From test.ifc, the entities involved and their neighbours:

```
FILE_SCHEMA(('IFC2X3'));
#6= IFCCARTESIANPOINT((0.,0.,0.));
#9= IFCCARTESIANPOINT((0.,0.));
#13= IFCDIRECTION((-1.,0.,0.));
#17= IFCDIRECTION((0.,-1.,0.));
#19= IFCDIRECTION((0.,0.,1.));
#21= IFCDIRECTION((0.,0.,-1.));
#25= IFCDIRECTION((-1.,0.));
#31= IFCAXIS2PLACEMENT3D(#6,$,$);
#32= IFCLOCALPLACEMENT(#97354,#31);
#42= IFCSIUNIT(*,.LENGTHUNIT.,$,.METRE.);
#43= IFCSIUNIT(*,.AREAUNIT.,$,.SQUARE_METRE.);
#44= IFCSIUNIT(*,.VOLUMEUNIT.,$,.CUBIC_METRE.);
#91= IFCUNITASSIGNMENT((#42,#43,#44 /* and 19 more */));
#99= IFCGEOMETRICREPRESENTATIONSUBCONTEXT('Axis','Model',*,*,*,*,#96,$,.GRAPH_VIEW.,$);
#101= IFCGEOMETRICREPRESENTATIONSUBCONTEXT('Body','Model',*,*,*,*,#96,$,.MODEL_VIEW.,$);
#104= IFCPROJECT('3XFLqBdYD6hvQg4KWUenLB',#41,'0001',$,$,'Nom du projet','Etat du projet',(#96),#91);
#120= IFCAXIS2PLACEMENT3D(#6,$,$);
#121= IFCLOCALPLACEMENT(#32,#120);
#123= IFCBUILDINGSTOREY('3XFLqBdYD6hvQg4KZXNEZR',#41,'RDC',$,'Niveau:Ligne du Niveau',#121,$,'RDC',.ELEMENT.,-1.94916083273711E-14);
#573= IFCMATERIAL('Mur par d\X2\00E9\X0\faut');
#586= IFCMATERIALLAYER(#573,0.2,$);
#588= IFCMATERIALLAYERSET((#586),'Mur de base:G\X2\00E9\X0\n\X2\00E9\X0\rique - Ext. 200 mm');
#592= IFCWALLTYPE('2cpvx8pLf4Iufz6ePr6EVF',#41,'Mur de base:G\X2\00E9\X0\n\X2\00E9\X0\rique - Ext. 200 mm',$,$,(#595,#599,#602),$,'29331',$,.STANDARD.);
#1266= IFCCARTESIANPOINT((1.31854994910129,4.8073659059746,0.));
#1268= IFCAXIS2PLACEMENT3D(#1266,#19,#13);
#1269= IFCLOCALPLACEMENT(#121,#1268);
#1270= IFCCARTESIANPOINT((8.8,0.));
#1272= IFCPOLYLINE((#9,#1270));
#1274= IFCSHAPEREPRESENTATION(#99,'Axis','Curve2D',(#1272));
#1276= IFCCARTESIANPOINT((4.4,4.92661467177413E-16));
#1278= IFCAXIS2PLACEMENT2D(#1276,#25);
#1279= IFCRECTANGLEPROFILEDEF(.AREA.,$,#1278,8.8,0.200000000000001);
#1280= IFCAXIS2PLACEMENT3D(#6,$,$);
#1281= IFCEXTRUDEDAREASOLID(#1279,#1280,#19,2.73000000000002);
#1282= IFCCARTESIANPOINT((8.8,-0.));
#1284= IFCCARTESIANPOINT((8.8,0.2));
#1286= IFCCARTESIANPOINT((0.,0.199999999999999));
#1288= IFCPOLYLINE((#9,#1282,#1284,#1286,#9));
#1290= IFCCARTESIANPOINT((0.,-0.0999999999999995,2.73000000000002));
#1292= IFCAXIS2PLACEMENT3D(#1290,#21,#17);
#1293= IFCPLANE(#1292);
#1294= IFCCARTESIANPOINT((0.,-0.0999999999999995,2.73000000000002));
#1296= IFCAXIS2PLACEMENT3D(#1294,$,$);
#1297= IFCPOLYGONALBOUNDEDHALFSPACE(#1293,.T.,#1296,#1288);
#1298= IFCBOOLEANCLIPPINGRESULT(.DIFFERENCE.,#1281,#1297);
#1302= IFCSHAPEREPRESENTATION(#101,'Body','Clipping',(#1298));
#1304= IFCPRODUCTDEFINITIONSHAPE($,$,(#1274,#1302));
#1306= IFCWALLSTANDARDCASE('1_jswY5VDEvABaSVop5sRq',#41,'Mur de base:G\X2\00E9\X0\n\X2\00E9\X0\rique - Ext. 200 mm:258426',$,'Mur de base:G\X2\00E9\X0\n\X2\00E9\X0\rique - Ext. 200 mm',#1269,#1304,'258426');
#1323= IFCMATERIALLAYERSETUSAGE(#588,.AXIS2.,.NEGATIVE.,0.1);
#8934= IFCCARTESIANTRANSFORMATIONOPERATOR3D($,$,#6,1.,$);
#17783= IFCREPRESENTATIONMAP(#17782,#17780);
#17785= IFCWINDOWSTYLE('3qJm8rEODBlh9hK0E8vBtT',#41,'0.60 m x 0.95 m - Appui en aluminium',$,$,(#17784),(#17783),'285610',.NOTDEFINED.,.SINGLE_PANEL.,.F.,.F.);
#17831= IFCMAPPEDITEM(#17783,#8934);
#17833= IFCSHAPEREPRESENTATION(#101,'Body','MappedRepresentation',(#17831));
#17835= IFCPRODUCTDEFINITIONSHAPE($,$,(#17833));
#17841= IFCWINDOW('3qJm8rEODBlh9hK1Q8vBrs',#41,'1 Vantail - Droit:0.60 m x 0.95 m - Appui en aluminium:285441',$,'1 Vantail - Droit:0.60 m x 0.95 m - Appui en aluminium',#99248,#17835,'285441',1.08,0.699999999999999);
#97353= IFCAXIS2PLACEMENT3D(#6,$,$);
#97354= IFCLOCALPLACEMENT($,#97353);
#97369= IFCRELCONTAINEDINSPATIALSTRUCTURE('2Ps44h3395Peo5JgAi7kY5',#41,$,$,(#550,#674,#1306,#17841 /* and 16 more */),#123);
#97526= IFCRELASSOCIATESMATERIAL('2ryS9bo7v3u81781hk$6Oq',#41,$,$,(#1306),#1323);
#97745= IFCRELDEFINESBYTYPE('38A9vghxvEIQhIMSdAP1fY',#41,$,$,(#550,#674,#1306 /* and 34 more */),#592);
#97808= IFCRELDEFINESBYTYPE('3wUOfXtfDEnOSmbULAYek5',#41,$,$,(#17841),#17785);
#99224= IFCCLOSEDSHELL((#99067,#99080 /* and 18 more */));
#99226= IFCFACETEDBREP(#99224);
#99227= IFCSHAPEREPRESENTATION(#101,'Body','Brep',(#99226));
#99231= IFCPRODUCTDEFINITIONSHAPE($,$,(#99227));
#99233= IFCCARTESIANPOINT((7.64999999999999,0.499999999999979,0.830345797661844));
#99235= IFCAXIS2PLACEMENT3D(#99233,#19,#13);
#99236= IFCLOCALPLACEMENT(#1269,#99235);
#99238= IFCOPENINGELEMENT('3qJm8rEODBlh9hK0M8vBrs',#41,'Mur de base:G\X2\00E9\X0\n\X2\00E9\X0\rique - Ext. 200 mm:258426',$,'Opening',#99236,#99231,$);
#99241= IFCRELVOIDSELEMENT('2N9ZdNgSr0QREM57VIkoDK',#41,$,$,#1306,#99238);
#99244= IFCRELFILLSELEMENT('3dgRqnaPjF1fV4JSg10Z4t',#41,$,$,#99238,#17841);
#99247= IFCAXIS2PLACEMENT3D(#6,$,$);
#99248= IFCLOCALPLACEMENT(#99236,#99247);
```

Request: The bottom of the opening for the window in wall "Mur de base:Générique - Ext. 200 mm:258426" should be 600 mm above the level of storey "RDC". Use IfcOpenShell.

```python
import numpy as np
import ifcopenshell
import ifcopenshell.api.geometry
import ifcopenshell.geom
import ifcopenshell.util.element
import ifcopenshell.util.placement
import ifcopenshell.util.shape
import ifcopenshell.util.unit

model = ifcopenshell.open("test.ifc")
unit_scale = ifcopenshell.util.unit.calculate_unit_scale(model)

window = model.by_guid("3qJm8rEODBlh9hK1Q8vBrs")
opening = window.FillsVoids[0].RelatingOpeningElement
storey = ifcopenshell.util.element.get_container(window, ifc_class="IfcBuildingStorey")
level = ifcopenshell.util.placement.get_local_placement(storey.ObjectPlacement)[2, 3]

# The opening's origin need not be at the sill, so measure its lowest point.
shape = ifcopenshell.geom.create_shape(ifcopenshell.geom.settings(), opening)
bottom = ifcopenshell.util.shape.get_shape_bottom_elevation(shape, shape.geometry) / unit_scale
dz = level + 0.6 - bottom

shift = np.array([0.0, 0.0, dz])
# The window is placed relative to its opening, so it follows when the opening moves.
matrix = ifcopenshell.util.placement.get_local_placement(opening.ObjectPlacement)
matrix[:3, 3] += shift
ifcopenshell.api.geometry.edit_object_placement(
    model, product=opening, matrix=matrix, is_si=False, should_transform_children=True
)

print(f"moved by {dz * unit_scale:+.3f} m")

model.write("test_rev.ifc")
```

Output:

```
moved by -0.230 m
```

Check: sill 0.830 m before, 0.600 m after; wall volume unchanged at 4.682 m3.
